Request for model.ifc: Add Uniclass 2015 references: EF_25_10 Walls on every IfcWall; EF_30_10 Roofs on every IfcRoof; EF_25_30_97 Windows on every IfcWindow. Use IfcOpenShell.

First a look at what the model holds.

```python
import ifcopenshell

model = ifcopenshell.open("model.ifc")
print(model.schema)
print("classifications:", [c.Name for c in model.by_type("IfcClassification")])
for ifc_class in ("IfcDoor", "IfcRoof", "IfcStair", "IfcWall", "IfcWindow"):
    print(ifc_class, len(model.by_type(ifc_class)))
```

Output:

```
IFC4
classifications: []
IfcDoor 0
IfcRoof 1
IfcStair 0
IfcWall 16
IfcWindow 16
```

```python
import ifcopenshell
import ifcopenshell.api.classification

model = ifcopenshell.open("model.ifc")

system = ifcopenshell.api.classification.add_classification(model, classification="Uniclass 2015")

codes = {
    "IfcWall": ("EF_25_10", "Walls"),
    "IfcRoof": ("EF_30_10", "Roofs"),
    "IfcWindow": ("EF_25_30_97", "Windows"),
}
for ifc_class, (code, name) in codes.items():
    products = model.by_type(ifc_class)
    ifcopenshell.api.classification.add_reference(
        model, products=products, classification=system, identification=code, name=name
    )
    print(code, len(products))

model.write("model_rev.ifc")
```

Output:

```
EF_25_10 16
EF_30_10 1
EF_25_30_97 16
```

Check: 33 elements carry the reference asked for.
